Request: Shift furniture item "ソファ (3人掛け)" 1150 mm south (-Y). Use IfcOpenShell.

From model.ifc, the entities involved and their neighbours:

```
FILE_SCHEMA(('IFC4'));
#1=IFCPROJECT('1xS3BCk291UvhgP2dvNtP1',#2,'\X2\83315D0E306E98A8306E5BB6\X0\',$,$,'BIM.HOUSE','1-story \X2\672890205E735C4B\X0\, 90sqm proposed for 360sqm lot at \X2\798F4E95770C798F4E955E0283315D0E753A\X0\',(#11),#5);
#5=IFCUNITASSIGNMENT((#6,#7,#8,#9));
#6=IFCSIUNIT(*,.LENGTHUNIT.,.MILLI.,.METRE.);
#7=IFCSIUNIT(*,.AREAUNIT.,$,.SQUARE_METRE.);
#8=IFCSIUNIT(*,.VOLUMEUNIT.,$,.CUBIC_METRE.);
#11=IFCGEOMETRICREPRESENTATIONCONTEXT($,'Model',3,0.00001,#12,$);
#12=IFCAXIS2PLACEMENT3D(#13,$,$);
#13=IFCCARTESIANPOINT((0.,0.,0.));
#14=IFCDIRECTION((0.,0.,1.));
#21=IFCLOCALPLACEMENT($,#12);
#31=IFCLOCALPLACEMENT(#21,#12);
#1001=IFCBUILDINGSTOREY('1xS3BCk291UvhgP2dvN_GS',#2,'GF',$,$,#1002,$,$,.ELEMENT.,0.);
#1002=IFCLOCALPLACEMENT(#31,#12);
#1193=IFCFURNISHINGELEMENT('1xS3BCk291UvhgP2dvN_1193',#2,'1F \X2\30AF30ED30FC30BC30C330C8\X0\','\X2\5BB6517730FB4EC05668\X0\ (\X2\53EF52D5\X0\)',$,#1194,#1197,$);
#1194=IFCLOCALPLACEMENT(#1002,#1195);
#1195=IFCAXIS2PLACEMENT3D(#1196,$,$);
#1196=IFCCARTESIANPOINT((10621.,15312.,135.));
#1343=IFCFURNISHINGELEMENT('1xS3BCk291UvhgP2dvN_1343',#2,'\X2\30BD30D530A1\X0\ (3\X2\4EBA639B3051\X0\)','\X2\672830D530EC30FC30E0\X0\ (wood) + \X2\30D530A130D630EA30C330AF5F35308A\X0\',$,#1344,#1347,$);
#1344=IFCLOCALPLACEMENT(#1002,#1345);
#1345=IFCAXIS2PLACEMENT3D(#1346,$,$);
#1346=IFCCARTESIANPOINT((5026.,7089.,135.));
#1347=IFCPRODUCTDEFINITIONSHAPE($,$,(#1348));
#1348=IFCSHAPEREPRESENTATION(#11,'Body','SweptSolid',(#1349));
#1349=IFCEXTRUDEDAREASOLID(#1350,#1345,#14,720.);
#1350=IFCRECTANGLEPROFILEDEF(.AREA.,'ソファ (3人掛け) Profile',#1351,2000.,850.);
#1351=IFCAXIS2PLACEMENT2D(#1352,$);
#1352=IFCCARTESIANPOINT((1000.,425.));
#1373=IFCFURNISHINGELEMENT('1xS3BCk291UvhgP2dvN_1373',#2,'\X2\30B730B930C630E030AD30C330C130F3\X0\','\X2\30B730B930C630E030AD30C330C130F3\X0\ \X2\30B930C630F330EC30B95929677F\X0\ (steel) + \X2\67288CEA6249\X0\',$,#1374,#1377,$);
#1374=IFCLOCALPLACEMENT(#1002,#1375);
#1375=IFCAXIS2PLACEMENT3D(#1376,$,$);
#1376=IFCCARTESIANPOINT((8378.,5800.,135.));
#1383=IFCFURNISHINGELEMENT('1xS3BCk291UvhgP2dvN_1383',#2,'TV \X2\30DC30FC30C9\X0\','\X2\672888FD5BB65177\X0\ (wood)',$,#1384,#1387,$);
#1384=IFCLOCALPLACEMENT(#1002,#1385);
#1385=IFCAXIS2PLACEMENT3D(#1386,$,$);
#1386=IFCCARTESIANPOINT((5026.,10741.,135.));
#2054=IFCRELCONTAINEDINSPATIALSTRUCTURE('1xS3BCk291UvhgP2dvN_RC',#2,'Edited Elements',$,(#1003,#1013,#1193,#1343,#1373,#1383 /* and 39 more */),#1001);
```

```python
import ifcopenshell
import ifcopenshell.api.geometry
import ifcopenshell.util.placement
import ifcopenshell.util.unit

model = ifcopenshell.open("model.ifc")
unit_scale = ifcopenshell.util.unit.calculate_unit_scale(model)

item = model.by_guid("1xS3BCk291UvhgP2dvN_1343")
matrix = ifcopenshell.util.placement.get_local_placement(item.ObjectPlacement)
matrix[1, 3] -= 1.15 / unit_scale
ifcopenshell.api.geometry.edit_object_placement(model, product=item, matrix=matrix, is_si=False)

print(ifcopenshell.util.placement.get_local_placement(item.ObjectPlacement).round(3) + 0.0)

model.write("model_updated.ifc")
```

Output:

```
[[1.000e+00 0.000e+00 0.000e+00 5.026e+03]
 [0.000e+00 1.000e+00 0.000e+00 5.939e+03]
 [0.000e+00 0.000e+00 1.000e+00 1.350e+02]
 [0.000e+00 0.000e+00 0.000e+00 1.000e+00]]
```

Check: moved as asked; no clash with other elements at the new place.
